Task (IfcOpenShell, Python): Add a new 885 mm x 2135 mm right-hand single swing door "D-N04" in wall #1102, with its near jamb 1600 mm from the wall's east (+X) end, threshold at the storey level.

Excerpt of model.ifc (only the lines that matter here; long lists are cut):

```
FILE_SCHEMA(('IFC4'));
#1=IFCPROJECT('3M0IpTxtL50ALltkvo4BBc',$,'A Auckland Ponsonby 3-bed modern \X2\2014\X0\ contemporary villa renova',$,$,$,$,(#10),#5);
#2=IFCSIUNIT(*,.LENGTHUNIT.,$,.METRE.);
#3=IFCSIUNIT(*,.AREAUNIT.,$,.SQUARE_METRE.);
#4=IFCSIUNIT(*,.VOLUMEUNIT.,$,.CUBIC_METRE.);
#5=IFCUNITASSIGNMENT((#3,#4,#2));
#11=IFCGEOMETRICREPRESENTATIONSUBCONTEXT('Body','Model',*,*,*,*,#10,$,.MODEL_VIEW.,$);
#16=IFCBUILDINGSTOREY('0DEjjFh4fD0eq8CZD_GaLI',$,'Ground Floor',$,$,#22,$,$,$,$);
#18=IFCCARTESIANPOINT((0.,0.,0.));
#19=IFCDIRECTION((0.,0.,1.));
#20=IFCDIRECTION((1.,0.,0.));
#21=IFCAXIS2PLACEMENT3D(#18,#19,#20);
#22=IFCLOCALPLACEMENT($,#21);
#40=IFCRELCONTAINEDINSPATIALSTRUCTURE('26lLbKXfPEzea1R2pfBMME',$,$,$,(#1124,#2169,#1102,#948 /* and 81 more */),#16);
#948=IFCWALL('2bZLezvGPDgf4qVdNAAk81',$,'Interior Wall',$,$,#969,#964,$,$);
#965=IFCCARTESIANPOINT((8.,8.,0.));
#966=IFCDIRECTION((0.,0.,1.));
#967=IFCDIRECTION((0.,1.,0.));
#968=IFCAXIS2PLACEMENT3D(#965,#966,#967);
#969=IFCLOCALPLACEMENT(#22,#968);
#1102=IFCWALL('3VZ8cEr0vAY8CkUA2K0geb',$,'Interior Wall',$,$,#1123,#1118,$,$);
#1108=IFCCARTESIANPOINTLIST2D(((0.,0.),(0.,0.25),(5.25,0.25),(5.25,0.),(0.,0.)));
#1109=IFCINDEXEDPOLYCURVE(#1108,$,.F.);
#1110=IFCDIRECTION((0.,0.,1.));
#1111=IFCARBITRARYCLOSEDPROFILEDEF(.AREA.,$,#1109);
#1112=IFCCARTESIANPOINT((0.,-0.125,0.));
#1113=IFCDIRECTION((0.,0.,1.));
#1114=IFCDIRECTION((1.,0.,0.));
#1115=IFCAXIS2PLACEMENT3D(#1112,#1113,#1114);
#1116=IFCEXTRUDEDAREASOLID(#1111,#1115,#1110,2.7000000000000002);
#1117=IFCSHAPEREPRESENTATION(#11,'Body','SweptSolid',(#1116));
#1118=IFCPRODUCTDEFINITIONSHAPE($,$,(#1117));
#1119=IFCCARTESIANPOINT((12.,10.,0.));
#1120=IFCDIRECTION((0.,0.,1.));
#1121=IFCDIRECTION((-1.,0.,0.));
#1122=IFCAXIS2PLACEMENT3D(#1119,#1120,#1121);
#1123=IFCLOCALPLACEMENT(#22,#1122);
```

```python
import numpy as np
import ifcopenshell
import ifcopenshell.api.feature
import ifcopenshell.api.geometry
import ifcopenshell.api.root
import ifcopenshell.api.spatial
import ifcopenshell.geom
import ifcopenshell.util.element
import ifcopenshell.util.placement
import ifcopenshell.util.representation
import ifcopenshell.util.shape
import ifcopenshell.util.unit

model = ifcopenshell.open("model.ifc")
unit_scale = ifcopenshell.util.unit.calculate_unit_scale(model)
settings = ifcopenshell.geom.settings()


def volume(element):
    """Net volume in cubic metres, openings subtracted."""
    shape = ifcopenshell.geom.create_shape(settings, element)
    return ifcopenshell.util.shape.get_volume(shape.geometry)


wall = model.by_guid("3VZ8cEr0vAY8CkUA2K0geb")
storey = ifcopenshell.util.element.get_container(wall, ifc_class="IfcBuildingStorey")
context = ifcopenshell.util.representation.get_context(model, "Model", "Body", "MODEL_VIEW")
before = volume(wall)

width, height, from_end, sill = 0.885, 2.135, 1.6, 0.0  # metres

# The wall runs along its own X axis, and the end named is its -X end.
wall_shape = ifcopenshell.geom.create_shape(settings, wall)
x, y, z = ifcopenshell.util.shape.get_vertices(wall_shape.geometry).T
start = x.min() + from_end
face, thickness = float(y.min()), float(y.max() - y.min())
wall_matrix = ifcopenshell.util.placement.get_local_placement(wall.ObjectPlacement)
level = ifcopenshell.util.placement.get_local_placement(storey.ObjectPlacement)[2, 3]


def in_wall(x, y):
    """Placement at x, y metres in the wall's axes, at sill height."""
    matrix = wall_matrix.copy()
    matrix[:, 3] = wall_matrix @ np.array([x / unit_scale, y / unit_scale, 0.0, 1.0])
    matrix[2, 3] = level + sill / unit_scale
    return matrix


# Opening: a box that overshoots both wall faces by 50 mm.
opening = ifcopenshell.api.root.create_entity(model, ifc_class="IfcOpeningElement", predefined_type="OPENING")
box = ifcopenshell.api.geometry.add_wall_representation(
    model, context=context, length=width, height=height, thickness=thickness + 0.1
)
ifcopenshell.api.geometry.assign_representation(model, product=opening, representation=box)
ifcopenshell.api.geometry.edit_object_placement(model, product=opening, matrix=in_wall(start, face - 0.05), is_si=False)
ifcopenshell.api.feature.add_feature(model, feature=opening, element=wall)

door = ifcopenshell.api.root.create_entity(model, ifc_class="IfcDoor", name="D-N04", predefined_type="DOOR")
door.OverallWidth, door.OverallHeight = width / unit_scale, height / unit_scale
door.OperationType = "SINGLE_SWING_RIGHT"
body = ifcopenshell.api.geometry.add_door_representation(
    model,
    context=context,
    overall_width=door.OverallWidth,
    overall_height=door.OverallHeight,
    operation_type="SINGLE_SWING_RIGHT",
    lining_properties={"LiningDepth": thickness / unit_scale, "ThresholdDepth": thickness / unit_scale},
)
ifcopenshell.api.geometry.assign_representation(model, product=door, representation=body)
ifcopenshell.api.spatial.assign_container(model, products=[door], relating_structure=storey)
ifcopenshell.api.feature.add_filling(model, opening=opening, element=door)

# The lining spans the wall, so the door starts at the wall face.
ifcopenshell.api.geometry.edit_object_placement(model, product=door, matrix=in_wall(start, face), is_si=False)

after = volume(wall)

print(f"wall volume {before:.3f} -> {after:.3f} m3")

model.write("model-out.ifc")
```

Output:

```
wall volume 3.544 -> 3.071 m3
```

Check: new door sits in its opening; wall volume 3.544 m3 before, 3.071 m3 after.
